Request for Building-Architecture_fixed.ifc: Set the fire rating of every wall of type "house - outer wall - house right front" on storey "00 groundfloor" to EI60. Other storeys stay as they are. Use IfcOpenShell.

First a look at what the model holds.

```python
import ifcopenshell
import ifcopenshell.util.element

model = ifcopenshell.open("Building-Architecture_fixed.ifc")
print(model.schema)
storey = next(s for s in model.by_type("IfcBuildingStorey") if s.Name == "00 groundfloor")
walls = [e for e in ifcopenshell.util.element.get_decomposition(storey) if e.is_a("IfcWall")]
seen = {}
for e in walls:
    element_type = ifcopenshell.util.element.get_type(e)
    key = (element_type.Name if element_type != e and element_type else None, ifcopenshell.util.element.get_pset(e, "Pset_WallCommon", "FireRating"))
    seen[key] = seen.get(key, 0) + 1
for (name, value), count in sorted(seen.items(), key=str):
    print(count, "x", name, "|", value)
```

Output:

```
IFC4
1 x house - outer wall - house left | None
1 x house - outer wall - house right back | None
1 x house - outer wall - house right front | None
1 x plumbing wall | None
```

```python
import ifcopenshell
import ifcopenshell.api.pset
import ifcopenshell.util.element

model = ifcopenshell.open("Building-Architecture_fixed.ifc")

storey = next(s for s in model.by_type("IfcBuildingStorey") if s.Name == "00 groundfloor")
walls = [e for e in ifcopenshell.util.element.get_decomposition(storey) if e.is_a("IfcWall")]

count = 0
for e in walls:
    element_type = ifcopenshell.util.element.get_type(e)
    if element_type in (None, e) or element_type.Name != "house - outer wall - house right front":
        continue
    # add_pset returns the element's existing set when there is one.
    pset = ifcopenshell.api.pset.add_pset(model, product=e, name="Pset_WallCommon")
    ifcopenshell.api.pset.edit_pset(model, pset=pset, properties={"FireRating": "EI60"})
    count += 1

print(count, "walls updated")

model.write("Building-Architecture_fixed_updated.ifc")
```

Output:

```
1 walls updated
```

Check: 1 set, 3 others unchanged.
